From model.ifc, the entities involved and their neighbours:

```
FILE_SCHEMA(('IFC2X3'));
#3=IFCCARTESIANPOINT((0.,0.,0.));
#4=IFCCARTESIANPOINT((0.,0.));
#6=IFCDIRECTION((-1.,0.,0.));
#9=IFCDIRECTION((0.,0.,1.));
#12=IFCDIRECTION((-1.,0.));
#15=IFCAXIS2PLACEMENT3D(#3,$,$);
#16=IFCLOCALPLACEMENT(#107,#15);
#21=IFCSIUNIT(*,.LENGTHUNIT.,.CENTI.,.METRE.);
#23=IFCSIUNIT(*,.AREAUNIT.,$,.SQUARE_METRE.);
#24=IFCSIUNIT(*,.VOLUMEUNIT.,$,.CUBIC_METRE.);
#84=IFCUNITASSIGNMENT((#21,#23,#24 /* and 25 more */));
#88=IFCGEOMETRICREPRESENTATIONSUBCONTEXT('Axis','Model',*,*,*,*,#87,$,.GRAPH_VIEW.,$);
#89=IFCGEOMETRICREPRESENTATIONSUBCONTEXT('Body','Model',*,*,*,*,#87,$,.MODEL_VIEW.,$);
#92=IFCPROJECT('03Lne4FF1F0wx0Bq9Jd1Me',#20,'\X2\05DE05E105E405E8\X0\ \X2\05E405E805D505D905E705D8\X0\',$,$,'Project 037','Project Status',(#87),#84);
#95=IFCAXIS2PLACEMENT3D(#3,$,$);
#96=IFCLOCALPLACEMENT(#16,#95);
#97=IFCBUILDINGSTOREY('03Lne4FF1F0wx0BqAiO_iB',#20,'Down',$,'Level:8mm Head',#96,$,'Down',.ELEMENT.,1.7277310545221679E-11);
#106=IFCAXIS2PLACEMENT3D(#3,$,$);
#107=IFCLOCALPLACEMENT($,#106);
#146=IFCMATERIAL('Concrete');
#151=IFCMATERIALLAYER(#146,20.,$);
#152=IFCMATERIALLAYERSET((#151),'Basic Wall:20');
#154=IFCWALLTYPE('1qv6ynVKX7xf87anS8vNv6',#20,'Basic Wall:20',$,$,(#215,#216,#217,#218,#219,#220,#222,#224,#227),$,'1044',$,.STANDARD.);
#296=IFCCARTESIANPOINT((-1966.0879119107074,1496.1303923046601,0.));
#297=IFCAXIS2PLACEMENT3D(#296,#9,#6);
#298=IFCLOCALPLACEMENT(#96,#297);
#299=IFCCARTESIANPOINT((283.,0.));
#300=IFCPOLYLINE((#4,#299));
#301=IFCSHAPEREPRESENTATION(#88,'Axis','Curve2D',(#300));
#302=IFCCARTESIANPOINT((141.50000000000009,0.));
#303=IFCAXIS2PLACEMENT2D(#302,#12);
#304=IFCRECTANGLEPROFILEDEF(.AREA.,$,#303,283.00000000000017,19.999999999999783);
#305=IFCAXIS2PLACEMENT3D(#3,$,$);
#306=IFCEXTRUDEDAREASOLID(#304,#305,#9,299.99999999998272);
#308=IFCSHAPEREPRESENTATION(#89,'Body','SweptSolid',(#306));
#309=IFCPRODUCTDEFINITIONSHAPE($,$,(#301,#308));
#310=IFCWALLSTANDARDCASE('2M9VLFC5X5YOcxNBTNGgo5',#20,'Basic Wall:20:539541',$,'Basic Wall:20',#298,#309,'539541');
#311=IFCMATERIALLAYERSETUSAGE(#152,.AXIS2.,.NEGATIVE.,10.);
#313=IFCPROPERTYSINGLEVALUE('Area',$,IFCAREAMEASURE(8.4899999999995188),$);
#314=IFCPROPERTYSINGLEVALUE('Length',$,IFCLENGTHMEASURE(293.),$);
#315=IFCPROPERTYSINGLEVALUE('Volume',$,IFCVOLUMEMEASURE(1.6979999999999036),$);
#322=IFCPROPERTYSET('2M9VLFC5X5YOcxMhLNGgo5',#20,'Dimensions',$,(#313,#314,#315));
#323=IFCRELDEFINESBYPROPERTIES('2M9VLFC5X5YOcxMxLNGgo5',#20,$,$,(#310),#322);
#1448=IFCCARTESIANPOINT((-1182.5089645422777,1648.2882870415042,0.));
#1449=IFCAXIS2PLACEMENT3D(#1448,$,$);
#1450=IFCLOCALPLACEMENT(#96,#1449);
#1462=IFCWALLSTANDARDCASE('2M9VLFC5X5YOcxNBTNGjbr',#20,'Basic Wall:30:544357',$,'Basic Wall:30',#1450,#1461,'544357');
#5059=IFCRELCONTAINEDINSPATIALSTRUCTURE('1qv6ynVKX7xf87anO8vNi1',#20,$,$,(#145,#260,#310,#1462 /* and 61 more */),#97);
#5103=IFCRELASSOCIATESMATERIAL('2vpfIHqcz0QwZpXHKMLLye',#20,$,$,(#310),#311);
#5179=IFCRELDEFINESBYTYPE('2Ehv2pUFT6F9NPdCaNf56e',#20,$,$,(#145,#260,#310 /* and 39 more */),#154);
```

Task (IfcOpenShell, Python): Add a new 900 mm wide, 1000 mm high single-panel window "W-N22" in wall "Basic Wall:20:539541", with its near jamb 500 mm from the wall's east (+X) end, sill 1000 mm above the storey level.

```python
import numpy as np
import ifcopenshell
import ifcopenshell.api.feature
import ifcopenshell.api.geometry
import ifcopenshell.api.pset
import ifcopenshell.api.root
import ifcopenshell.api.spatial
import ifcopenshell.api.type
import ifcopenshell.geom
import ifcopenshell.util.element
import ifcopenshell.util.placement
import ifcopenshell.util.representation
import ifcopenshell.util.shape
import ifcopenshell.util.unit

model = ifcopenshell.open("model.ifc")
unit_scale = ifcopenshell.util.unit.calculate_unit_scale(model)
area_scale = ifcopenshell.util.unit.calculate_unit_scale(model, "AREAUNIT")
volume_scale = ifcopenshell.util.unit.calculate_unit_scale(model, "VOLUMEUNIT")
settings = ifcopenshell.geom.settings()


def volume(element):
    """Net volume in cubic metres, openings subtracted."""
    shape = ifcopenshell.geom.create_shape(settings, element)
    return ifcopenshell.util.shape.get_volume(shape.geometry)


wall = model.by_id(310)
storey = ifcopenshell.util.element.get_container(wall, ifc_class="IfcBuildingStorey")
context = ifcopenshell.util.representation.get_context(model, "Model", "Body", "MODEL_VIEW")
before = volume(wall)

width, height, from_end, sill = 0.9, 1, 0.5, 1  # metres

# The wall runs along its own X axis, and the end named is its -X end.
wall_shape = ifcopenshell.geom.create_shape(settings, wall)
x, y, z = ifcopenshell.util.shape.get_vertices(wall_shape.geometry).T
start = x.min() + from_end
face, thickness = float(y.min()), float(y.max() - y.min())
wall_matrix = ifcopenshell.util.placement.get_local_placement(wall.ObjectPlacement)
level = ifcopenshell.util.placement.get_local_placement(storey.ObjectPlacement)[2, 3]


def in_wall(x, y):
    """Placement at x, y metres in the wall's axes, at sill height."""
    matrix = wall_matrix.copy()
    matrix[:, 3] = wall_matrix @ np.array([x / unit_scale, y / unit_scale, 0.0, 1.0])
    matrix[2, 3] = level + sill / unit_scale
    return matrix


# Opening: a box that overshoots both wall faces by 50 mm.
opening = ifcopenshell.api.root.create_entity(model, ifc_class="IfcOpeningElement")
box = ifcopenshell.api.geometry.add_wall_representation(
    model, context=context, length=width, height=height, thickness=thickness + 0.1
)
ifcopenshell.api.geometry.assign_representation(model, product=opening, representation=box)
ifcopenshell.api.geometry.edit_object_placement(model, product=opening, matrix=in_wall(start, face - 0.05), is_si=False)
ifcopenshell.api.feature.add_feature(model, feature=opening, element=wall)

window = ifcopenshell.api.root.create_entity(model, ifc_class="IfcWindow", name="W-N22")
window.OverallWidth, window.OverallHeight = width / unit_scale, height / unit_scale
body = ifcopenshell.api.geometry.add_window_representation(
    model,
    context=context,
    overall_width=window.OverallWidth,
    overall_height=window.OverallHeight,
    partition_type="SINGLE_PANEL",
)
ifcopenshell.api.geometry.assign_representation(model, product=window, representation=body)
ifcopenshell.api.spatial.assign_container(model, products=[window], relating_structure=storey)
fills = ifcopenshell.api.feature.add_filling(model, opening=opening, element=window)
fills.OwnerHistory = window.OwnerHistory  # required in IFC2X3

# IFC2X3 keeps the operation on the window style.
style = ifcopenshell.api.root.create_entity(model, ifc_class="IfcWindowStyle", name="W-N22")
style.OperationType, style.ConstructionType = "SINGLE_PANEL", "NOTDEFINED"
style.ParameterTakesPrecedence = style.Sizeable = False
ifcopenshell.api.type.assign_type(model, related_objects=[window], relating_type=style)

# Centre the window in the wall's thickness.
ifcopenshell.api.geometry.edit_object_placement(model, product=window, matrix=in_wall(start, face), is_si=False)
window_shape = ifcopenshell.geom.create_shape(settings, window)
depth = ifcopenshell.util.shape.get_vertices(window_shape.geometry)[:, 1]
offset = face + thickness / 2 - (depth.min() + depth.max()) / 2
ifcopenshell.api.geometry.edit_object_placement(model, product=window, matrix=in_wall(start, offset), is_si=False)

after = volume(wall)

# Update the wall's stored quantities.
pset = model.by_id(ifcopenshell.util.element.get_pset(wall, "Dimensions", should_inherit=False)["id"])
ifcopenshell.api.pset.edit_pset(model, pset=pset, properties={
    "Area": model.create_entity("IfcAreaMeasure", after / thickness / area_scale),
    "Volume": model.create_entity("IfcVolumeMeasure", after / volume_scale),
})

print(f"wall volume {before:.3f} -> {after:.3f} m3")

model.write("model_v2.ifc")
```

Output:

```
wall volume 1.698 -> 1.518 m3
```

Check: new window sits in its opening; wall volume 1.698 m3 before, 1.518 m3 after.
